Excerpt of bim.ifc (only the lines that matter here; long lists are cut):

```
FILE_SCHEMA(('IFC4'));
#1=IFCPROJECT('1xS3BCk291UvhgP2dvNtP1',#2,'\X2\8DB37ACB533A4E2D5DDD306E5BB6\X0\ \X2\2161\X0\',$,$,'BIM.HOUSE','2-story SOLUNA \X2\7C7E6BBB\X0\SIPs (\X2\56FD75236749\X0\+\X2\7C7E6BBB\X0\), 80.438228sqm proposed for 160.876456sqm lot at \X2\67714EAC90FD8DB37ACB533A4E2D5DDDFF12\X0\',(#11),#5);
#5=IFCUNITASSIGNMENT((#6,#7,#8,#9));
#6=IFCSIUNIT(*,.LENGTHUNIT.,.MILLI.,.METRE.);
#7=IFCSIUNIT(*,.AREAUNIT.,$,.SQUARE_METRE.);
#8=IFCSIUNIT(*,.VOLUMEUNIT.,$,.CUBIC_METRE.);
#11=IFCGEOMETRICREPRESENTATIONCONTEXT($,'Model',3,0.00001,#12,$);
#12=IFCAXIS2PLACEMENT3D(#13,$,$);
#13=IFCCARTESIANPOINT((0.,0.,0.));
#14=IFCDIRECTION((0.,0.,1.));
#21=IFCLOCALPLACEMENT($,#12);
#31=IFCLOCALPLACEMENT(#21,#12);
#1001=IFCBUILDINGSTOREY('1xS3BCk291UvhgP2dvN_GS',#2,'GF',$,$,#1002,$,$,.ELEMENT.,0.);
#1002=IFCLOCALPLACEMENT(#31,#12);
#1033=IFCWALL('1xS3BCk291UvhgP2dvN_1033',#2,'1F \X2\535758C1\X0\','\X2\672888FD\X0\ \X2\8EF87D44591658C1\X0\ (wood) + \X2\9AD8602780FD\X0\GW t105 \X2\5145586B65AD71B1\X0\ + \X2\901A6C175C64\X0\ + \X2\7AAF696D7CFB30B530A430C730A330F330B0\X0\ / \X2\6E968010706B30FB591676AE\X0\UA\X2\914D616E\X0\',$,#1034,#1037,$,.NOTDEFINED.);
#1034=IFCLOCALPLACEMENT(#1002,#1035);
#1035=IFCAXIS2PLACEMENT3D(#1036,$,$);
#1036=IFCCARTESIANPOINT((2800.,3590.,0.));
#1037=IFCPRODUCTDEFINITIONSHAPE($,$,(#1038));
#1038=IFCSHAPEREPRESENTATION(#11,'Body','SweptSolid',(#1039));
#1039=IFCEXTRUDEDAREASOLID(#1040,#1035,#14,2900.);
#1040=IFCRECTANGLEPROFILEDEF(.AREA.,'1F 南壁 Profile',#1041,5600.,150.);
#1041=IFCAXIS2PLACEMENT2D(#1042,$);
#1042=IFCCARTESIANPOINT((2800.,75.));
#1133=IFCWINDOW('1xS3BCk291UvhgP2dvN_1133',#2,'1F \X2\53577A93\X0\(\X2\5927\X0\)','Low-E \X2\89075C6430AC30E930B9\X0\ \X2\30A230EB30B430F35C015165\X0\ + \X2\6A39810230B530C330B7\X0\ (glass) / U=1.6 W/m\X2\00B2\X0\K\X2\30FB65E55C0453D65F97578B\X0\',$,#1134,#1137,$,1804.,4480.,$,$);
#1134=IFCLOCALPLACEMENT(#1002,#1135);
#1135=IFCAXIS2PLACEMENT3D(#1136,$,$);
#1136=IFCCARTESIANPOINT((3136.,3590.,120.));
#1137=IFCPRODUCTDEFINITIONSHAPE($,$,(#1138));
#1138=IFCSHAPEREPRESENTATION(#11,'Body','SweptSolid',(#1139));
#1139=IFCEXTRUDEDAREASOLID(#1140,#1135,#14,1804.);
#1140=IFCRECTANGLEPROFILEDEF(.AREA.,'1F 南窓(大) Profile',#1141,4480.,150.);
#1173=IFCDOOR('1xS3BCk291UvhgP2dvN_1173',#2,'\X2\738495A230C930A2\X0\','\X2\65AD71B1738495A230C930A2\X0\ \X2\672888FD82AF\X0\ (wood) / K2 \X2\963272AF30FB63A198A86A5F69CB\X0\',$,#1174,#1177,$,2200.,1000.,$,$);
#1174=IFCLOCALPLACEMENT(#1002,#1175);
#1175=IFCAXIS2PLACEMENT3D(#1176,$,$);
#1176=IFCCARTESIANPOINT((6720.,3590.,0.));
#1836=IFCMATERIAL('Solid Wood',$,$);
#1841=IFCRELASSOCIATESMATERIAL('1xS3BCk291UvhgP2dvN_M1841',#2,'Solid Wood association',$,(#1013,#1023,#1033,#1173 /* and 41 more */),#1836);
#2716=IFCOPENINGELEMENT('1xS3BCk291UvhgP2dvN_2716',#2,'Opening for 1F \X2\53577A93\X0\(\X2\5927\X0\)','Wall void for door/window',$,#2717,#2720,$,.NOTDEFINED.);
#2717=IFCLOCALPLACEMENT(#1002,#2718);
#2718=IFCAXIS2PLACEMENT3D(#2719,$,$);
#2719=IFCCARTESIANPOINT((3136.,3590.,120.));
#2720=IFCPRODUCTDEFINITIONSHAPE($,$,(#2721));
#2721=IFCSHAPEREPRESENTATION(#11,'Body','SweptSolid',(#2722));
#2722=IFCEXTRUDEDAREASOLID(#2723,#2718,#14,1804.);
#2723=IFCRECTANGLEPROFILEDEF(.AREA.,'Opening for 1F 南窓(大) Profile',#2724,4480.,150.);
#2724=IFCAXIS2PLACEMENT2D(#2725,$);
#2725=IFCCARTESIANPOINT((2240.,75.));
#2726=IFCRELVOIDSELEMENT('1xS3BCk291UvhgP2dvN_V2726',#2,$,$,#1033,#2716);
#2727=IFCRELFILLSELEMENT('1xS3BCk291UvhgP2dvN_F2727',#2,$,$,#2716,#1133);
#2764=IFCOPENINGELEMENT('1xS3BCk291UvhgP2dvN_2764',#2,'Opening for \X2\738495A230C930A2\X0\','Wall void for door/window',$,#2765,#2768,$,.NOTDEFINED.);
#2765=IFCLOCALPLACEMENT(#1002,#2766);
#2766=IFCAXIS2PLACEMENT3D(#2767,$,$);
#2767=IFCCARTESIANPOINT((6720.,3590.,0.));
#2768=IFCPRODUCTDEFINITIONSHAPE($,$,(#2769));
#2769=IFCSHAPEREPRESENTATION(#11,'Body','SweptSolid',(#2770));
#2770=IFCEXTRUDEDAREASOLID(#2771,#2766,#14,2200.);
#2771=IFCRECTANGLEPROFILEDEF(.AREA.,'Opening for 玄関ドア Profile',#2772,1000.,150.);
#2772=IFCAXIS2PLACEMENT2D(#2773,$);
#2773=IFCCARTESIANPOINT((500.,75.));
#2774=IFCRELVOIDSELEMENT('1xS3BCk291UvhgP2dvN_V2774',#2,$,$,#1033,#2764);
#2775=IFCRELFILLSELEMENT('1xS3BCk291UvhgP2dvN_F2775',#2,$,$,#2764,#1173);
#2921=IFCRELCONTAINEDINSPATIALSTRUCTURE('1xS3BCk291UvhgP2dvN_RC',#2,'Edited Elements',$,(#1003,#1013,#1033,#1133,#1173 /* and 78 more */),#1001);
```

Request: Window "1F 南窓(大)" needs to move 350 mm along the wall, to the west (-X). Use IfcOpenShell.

```python
import ifcopenshell
import ifcopenshell.api.geometry
import ifcopenshell.util.placement

model = ifcopenshell.open("bim.ifc")

window = model.by_guid("1xS3BCk291UvhgP2dvN_1133")
opening = window.FillsVoids[0].RelatingOpeningElement
wall = opening.VoidsElements[0].RelatingBuildingElement

wall_matrix = ifcopenshell.util.placement.get_local_placement(wall.ObjectPlacement)
shift = wall_matrix[:3, 0] * -350.0
before = ifcopenshell.util.placement.get_local_placement(window.ObjectPlacement)[:3, 3].copy()

# The window is not placed relative to its opening, so move both.
for product in (opening, window):
    matrix = ifcopenshell.util.placement.get_local_placement(product.ObjectPlacement)
    matrix[:3, 3] += shift
    ifcopenshell.api.geometry.edit_object_placement(model, product=product, matrix=matrix, is_si=False)

after = ifcopenshell.util.placement.get_local_placement(window.ObjectPlacement)[:3, 3]
print("window moved by", (after - before).round(3) + 0.0)

model.write("bim_v2.ifc")
```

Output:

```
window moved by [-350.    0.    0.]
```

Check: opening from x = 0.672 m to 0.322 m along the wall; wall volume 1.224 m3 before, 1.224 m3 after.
